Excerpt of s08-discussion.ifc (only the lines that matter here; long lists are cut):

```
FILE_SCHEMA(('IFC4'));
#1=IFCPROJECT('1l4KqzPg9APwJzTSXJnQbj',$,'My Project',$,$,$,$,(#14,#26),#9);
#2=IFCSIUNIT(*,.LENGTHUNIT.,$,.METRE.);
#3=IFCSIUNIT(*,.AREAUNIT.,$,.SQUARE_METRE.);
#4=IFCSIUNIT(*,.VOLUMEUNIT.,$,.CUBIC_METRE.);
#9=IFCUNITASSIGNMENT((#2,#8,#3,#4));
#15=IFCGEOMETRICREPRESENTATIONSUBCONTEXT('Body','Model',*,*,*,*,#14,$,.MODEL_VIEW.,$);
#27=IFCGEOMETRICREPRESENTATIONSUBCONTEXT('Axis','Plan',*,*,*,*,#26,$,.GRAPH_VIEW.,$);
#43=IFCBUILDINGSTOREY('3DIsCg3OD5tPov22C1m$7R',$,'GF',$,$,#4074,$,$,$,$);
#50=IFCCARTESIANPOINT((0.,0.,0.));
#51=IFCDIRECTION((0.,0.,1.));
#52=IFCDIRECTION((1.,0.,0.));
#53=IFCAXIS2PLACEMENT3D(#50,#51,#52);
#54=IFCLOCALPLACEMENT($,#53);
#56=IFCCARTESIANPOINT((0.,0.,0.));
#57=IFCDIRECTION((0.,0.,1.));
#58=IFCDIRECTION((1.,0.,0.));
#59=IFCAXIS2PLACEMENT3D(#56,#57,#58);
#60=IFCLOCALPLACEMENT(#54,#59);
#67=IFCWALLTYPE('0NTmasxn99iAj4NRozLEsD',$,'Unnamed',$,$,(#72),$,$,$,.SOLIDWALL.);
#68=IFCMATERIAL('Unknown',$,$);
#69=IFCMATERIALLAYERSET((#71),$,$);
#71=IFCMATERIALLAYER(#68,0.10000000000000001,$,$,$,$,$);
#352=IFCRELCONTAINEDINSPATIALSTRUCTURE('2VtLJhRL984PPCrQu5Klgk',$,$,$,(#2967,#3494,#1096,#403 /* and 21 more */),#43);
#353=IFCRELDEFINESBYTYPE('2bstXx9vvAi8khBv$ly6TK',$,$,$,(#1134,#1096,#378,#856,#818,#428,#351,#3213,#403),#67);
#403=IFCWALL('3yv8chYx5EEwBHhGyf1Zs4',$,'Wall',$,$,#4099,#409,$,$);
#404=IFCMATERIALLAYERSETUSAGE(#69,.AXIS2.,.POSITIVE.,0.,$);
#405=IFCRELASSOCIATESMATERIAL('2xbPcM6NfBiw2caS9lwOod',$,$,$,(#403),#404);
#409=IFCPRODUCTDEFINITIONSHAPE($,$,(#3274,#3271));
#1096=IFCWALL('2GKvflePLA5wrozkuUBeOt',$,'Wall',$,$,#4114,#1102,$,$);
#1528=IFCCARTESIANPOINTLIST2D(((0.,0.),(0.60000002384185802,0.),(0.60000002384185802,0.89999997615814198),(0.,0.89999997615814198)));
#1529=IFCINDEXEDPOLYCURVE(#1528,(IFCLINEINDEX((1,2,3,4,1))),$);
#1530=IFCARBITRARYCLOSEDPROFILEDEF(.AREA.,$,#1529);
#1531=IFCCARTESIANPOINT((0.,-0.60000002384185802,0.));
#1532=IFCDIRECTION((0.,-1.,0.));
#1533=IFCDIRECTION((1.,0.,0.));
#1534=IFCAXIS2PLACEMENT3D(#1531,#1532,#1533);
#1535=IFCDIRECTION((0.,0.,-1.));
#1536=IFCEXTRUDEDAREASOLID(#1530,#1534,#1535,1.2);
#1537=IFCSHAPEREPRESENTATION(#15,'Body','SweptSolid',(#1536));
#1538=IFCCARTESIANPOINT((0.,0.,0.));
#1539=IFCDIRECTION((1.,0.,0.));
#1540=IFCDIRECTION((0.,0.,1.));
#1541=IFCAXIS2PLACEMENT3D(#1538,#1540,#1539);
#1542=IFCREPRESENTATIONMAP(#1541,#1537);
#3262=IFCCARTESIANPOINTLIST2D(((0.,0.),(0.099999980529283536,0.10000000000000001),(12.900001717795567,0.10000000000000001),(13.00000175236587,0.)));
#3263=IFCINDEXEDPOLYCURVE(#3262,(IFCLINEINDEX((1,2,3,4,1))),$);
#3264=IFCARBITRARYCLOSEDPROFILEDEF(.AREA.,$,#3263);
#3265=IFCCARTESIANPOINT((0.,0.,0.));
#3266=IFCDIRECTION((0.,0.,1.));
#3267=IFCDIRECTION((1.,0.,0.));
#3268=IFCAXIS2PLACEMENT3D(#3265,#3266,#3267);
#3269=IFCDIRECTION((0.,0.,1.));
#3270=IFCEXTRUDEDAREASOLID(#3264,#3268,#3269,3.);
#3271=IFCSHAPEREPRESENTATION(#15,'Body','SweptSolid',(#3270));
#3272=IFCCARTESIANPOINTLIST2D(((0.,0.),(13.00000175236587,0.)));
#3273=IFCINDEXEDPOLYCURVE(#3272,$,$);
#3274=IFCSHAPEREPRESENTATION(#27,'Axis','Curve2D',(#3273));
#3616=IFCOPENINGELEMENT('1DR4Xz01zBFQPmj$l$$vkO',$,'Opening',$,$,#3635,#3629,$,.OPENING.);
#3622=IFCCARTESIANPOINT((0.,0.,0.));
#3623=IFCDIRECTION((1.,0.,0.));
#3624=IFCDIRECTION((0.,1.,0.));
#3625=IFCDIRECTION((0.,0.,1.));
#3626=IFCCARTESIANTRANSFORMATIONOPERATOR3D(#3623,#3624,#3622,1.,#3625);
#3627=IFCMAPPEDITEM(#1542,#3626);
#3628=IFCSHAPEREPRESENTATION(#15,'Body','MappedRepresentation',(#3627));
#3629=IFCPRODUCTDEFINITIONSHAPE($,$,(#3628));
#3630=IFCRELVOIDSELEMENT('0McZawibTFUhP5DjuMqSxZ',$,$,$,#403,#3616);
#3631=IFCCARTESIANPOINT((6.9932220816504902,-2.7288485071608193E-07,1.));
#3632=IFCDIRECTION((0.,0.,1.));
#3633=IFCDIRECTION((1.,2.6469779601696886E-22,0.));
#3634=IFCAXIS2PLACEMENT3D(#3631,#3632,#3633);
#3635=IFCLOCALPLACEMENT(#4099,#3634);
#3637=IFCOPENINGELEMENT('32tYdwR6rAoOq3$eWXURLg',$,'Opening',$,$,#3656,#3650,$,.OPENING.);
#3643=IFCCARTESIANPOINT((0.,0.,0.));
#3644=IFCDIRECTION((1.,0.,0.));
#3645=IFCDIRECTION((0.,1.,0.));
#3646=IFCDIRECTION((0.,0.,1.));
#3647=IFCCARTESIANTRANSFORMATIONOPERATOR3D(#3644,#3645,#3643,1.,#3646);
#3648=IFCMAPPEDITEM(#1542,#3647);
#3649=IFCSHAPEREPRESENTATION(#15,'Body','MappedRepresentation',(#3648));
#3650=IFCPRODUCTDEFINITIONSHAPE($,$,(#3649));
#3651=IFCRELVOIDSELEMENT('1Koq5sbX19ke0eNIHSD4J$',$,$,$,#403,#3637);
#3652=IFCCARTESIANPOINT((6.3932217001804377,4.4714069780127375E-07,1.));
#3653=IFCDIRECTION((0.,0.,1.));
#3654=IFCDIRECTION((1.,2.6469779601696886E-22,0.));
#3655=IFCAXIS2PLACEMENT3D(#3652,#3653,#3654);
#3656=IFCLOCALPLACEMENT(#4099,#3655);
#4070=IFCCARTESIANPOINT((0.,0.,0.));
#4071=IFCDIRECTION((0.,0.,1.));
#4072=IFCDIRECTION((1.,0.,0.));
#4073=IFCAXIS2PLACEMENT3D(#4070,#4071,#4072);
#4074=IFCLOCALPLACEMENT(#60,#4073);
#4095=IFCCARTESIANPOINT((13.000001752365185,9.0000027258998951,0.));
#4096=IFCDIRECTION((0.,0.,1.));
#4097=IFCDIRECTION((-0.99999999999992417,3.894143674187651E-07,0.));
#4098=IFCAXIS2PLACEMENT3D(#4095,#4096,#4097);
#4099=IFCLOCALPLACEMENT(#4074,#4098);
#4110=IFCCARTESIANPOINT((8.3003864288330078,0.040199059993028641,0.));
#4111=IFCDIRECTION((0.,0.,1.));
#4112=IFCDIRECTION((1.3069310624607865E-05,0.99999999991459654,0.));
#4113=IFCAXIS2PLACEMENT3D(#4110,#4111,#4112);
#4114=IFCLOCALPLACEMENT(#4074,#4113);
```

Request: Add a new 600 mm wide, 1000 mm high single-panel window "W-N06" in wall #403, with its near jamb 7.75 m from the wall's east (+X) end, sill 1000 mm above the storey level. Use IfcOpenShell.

```python
import numpy as np
import ifcopenshell
import ifcopenshell.api.feature
import ifcopenshell.api.geometry
import ifcopenshell.api.root
import ifcopenshell.api.spatial
import ifcopenshell.geom
import ifcopenshell.util.element
import ifcopenshell.util.placement
import ifcopenshell.util.representation
import ifcopenshell.util.shape
import ifcopenshell.util.unit

model = ifcopenshell.open("s08-discussion.ifc")
unit_scale = ifcopenshell.util.unit.calculate_unit_scale(model)
settings = ifcopenshell.geom.settings()


def volume(element):
    """Net volume in cubic metres, openings subtracted."""
    shape = ifcopenshell.geom.create_shape(settings, element)
    return ifcopenshell.util.shape.get_volume(shape.geometry)


wall = model.by_id(403)
storey = ifcopenshell.util.element.get_container(wall, ifc_class="IfcBuildingStorey")
context = ifcopenshell.util.representation.get_context(model, "Model", "Body", "MODEL_VIEW")
before = volume(wall)

width, height, from_end, sill = 0.6, 1, 7.75, 1  # metres

# The wall runs along its own X axis, and the end named is its -X end.
wall_shape = ifcopenshell.geom.create_shape(settings, wall)
x, y, z = ifcopenshell.util.shape.get_vertices(wall_shape.geometry).T
start = x.min() + from_end
face, thickness = float(y.min()), float(y.max() - y.min())
wall_matrix = ifcopenshell.util.placement.get_local_placement(wall.ObjectPlacement)
level = ifcopenshell.util.placement.get_local_placement(storey.ObjectPlacement)[2, 3]


def in_wall(x, y):
    """Placement at x, y metres in the wall's axes, at sill height."""
    matrix = wall_matrix.copy()
    matrix[:, 3] = wall_matrix @ np.array([x / unit_scale, y / unit_scale, 0.0, 1.0])
    matrix[2, 3] = level + sill / unit_scale
    return matrix


# Opening: a box that overshoots both wall faces by 50 mm.
opening = ifcopenshell.api.root.create_entity(model, ifc_class="IfcOpeningElement", predefined_type="OPENING")
box = ifcopenshell.api.geometry.add_wall_representation(
    model, context=context, length=width, height=height, thickness=thickness + 0.1
)
ifcopenshell.api.geometry.assign_representation(model, product=opening, representation=box)
ifcopenshell.api.geometry.edit_object_placement(model, product=opening, matrix=in_wall(start, face - 0.05), is_si=False)
ifcopenshell.api.feature.add_feature(model, feature=opening, element=wall)

window = ifcopenshell.api.root.create_entity(model, ifc_class="IfcWindow", name="W-N06", predefined_type="WINDOW")
window.OverallWidth, window.OverallHeight = width / unit_scale, height / unit_scale
window.PartitioningType = "SINGLE_PANEL"
body = ifcopenshell.api.geometry.add_window_representation(
    model,
    context=context,
    overall_width=window.OverallWidth,
    overall_height=window.OverallHeight,
    partition_type="SINGLE_PANEL",
)
ifcopenshell.api.geometry.assign_representation(model, product=window, representation=body)
ifcopenshell.api.spatial.assign_container(model, products=[window], relating_structure=storey)
ifcopenshell.api.feature.add_filling(model, opening=opening, element=window)

# Centre the window in the wall's thickness.
ifcopenshell.api.geometry.edit_object_placement(model, product=window, matrix=in_wall(start, face), is_si=False)
window_shape = ifcopenshell.geom.create_shape(settings, window)
depth = ifcopenshell.util.shape.get_vertices(window_shape.geometry)[:, 1]
offset = face + thickness / 2 - (depth.min() + depth.max()) / 2
ifcopenshell.api.geometry.edit_object_placement(model, product=window, matrix=in_wall(start, offset), is_si=False)

after = volume(wall)

print(f"wall volume {before:.3f} -> {after:.3f} m3")

model.write("s08-discussion_rev.ifc")
```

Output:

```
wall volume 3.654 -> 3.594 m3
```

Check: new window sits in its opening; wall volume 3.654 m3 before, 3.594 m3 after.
